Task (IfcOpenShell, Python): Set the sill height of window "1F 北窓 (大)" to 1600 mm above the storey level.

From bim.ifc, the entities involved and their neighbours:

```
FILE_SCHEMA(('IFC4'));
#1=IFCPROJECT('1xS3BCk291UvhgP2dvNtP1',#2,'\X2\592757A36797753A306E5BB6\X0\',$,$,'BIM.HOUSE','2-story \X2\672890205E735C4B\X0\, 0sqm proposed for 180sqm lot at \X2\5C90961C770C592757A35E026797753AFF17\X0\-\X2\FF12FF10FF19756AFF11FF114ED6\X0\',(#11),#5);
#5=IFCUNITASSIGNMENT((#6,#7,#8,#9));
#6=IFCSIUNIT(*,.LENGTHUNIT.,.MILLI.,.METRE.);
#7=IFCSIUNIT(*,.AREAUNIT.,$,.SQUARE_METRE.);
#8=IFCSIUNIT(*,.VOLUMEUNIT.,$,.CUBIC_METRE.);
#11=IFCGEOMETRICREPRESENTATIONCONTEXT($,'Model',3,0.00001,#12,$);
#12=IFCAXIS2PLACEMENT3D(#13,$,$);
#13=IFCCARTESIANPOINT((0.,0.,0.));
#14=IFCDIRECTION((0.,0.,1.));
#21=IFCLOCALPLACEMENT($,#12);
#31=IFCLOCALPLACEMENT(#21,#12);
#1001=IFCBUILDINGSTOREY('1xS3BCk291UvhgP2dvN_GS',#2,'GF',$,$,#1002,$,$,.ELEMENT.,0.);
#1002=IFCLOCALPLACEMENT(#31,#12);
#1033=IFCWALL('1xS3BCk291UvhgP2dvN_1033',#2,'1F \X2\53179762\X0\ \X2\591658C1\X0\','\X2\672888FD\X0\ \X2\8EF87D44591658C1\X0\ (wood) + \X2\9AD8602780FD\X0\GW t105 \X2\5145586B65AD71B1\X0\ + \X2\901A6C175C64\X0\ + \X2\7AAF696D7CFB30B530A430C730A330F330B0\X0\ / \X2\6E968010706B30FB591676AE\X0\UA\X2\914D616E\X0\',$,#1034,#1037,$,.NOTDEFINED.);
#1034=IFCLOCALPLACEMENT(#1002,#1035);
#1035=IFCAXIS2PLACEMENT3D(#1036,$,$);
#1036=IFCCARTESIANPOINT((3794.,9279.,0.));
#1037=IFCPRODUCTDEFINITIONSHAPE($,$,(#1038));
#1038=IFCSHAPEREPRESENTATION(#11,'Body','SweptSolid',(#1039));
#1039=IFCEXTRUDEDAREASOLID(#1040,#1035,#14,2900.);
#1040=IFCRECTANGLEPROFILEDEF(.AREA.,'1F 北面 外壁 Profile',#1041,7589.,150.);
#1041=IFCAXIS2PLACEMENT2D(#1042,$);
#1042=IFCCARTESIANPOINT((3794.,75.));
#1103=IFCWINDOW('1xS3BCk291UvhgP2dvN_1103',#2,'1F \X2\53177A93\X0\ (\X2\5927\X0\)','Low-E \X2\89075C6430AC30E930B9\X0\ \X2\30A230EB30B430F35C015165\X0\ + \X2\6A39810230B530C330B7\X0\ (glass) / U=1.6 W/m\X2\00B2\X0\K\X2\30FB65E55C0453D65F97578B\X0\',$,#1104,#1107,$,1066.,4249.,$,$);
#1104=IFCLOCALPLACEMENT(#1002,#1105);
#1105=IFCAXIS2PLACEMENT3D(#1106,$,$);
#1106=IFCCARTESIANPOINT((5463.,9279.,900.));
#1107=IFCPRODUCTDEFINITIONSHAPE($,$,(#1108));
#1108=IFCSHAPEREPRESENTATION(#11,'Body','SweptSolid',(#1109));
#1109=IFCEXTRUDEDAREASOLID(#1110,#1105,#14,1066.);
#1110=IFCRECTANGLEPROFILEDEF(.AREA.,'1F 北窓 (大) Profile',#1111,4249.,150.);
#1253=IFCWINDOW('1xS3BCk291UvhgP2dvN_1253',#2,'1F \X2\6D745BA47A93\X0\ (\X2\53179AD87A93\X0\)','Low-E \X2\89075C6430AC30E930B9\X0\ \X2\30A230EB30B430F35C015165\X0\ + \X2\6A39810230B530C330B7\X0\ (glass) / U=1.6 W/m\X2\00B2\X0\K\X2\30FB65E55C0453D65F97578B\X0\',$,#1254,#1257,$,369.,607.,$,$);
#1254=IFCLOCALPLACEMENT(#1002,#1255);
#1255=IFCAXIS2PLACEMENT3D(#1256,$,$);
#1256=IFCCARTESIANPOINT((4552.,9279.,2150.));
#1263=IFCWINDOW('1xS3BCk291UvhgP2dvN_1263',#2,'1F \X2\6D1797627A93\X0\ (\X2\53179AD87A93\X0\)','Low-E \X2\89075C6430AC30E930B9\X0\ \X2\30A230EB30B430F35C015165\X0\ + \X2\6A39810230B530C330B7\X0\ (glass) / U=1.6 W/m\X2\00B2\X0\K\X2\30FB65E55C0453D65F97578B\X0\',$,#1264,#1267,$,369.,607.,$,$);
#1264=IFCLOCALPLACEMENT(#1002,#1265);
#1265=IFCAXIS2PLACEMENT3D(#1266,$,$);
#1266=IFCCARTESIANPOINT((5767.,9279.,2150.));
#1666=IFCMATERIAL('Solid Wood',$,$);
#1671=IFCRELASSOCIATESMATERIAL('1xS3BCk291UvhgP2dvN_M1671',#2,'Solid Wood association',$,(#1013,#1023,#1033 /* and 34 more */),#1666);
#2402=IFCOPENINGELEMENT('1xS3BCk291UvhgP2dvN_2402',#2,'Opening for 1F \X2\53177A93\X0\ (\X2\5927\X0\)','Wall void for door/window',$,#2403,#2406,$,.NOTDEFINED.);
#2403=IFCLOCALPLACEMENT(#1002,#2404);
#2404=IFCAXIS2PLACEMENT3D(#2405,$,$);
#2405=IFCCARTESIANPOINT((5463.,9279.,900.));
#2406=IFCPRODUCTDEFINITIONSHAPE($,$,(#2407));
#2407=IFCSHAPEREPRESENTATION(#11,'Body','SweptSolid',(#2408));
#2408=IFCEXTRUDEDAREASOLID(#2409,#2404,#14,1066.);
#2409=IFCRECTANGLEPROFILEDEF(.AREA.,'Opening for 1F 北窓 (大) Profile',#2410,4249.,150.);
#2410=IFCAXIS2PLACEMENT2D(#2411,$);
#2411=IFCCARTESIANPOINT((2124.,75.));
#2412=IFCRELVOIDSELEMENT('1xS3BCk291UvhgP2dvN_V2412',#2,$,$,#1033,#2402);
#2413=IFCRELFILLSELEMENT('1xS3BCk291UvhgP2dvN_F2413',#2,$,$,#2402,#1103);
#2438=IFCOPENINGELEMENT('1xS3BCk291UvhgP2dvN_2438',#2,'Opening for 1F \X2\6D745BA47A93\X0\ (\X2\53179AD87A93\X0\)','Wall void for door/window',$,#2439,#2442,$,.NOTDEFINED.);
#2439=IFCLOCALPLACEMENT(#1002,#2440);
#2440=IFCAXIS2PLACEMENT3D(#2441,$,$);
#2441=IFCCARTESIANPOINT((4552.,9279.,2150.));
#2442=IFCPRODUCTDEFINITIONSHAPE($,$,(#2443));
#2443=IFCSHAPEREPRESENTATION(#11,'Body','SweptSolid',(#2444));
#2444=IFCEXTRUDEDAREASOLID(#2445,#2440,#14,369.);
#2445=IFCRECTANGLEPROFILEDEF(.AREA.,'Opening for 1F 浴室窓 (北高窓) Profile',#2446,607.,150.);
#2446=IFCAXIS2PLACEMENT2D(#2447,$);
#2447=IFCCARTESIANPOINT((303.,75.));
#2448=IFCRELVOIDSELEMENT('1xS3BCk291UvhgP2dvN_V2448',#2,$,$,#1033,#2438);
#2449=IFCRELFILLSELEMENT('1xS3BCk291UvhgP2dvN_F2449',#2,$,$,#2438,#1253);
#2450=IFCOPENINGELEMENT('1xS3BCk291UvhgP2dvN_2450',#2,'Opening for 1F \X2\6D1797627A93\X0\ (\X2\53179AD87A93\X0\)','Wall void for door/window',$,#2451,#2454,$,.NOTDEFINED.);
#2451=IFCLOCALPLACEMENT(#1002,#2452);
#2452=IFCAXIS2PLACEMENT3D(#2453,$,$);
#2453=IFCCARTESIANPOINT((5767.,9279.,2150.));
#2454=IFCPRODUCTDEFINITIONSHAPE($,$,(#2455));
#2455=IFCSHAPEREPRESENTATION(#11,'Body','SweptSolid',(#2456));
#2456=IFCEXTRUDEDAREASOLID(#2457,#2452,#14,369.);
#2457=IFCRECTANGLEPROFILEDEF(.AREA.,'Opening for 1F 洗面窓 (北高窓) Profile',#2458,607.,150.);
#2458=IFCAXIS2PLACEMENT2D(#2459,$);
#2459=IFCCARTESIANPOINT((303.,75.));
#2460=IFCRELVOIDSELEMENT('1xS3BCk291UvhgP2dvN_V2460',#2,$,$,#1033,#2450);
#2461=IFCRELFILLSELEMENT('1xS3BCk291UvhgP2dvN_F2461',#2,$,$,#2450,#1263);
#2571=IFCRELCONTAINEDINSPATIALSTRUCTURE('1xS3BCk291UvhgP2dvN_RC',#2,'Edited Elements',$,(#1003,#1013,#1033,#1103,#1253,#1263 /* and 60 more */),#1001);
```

```python
import numpy as np
import ifcopenshell
import ifcopenshell.api.geometry
import ifcopenshell.geom
import ifcopenshell.util.element
import ifcopenshell.util.placement
import ifcopenshell.util.shape
import ifcopenshell.util.unit

model = ifcopenshell.open("bim.ifc")
unit_scale = ifcopenshell.util.unit.calculate_unit_scale(model)

window = model.by_guid("1xS3BCk291UvhgP2dvN_1103")
opening = window.FillsVoids[0].RelatingOpeningElement
storey = ifcopenshell.util.element.get_container(window, ifc_class="IfcBuildingStorey")
level = ifcopenshell.util.placement.get_local_placement(storey.ObjectPlacement)[2, 3]

# The opening's origin need not be at the sill, so measure its lowest point.
shape = ifcopenshell.geom.create_shape(ifcopenshell.geom.settings(), opening)
bottom = ifcopenshell.util.shape.get_shape_bottom_elevation(shape, shape.geometry) / unit_scale
dz = level + 1.6 / unit_scale - bottom

shift = np.array([0.0, 0.0, dz])
# The window is not placed relative to its opening, so move both.
for product in (opening, window):
    matrix = ifcopenshell.util.placement.get_local_placement(product.ObjectPlacement)
    matrix[:3, 3] += shift
    ifcopenshell.api.geometry.edit_object_placement(model, product=product, matrix=matrix, is_si=False)

print(f"moved by {dz * unit_scale:+.3f} m")

model.write("bim_v2.ifc")
```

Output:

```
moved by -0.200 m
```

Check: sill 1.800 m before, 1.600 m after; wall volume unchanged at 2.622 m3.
